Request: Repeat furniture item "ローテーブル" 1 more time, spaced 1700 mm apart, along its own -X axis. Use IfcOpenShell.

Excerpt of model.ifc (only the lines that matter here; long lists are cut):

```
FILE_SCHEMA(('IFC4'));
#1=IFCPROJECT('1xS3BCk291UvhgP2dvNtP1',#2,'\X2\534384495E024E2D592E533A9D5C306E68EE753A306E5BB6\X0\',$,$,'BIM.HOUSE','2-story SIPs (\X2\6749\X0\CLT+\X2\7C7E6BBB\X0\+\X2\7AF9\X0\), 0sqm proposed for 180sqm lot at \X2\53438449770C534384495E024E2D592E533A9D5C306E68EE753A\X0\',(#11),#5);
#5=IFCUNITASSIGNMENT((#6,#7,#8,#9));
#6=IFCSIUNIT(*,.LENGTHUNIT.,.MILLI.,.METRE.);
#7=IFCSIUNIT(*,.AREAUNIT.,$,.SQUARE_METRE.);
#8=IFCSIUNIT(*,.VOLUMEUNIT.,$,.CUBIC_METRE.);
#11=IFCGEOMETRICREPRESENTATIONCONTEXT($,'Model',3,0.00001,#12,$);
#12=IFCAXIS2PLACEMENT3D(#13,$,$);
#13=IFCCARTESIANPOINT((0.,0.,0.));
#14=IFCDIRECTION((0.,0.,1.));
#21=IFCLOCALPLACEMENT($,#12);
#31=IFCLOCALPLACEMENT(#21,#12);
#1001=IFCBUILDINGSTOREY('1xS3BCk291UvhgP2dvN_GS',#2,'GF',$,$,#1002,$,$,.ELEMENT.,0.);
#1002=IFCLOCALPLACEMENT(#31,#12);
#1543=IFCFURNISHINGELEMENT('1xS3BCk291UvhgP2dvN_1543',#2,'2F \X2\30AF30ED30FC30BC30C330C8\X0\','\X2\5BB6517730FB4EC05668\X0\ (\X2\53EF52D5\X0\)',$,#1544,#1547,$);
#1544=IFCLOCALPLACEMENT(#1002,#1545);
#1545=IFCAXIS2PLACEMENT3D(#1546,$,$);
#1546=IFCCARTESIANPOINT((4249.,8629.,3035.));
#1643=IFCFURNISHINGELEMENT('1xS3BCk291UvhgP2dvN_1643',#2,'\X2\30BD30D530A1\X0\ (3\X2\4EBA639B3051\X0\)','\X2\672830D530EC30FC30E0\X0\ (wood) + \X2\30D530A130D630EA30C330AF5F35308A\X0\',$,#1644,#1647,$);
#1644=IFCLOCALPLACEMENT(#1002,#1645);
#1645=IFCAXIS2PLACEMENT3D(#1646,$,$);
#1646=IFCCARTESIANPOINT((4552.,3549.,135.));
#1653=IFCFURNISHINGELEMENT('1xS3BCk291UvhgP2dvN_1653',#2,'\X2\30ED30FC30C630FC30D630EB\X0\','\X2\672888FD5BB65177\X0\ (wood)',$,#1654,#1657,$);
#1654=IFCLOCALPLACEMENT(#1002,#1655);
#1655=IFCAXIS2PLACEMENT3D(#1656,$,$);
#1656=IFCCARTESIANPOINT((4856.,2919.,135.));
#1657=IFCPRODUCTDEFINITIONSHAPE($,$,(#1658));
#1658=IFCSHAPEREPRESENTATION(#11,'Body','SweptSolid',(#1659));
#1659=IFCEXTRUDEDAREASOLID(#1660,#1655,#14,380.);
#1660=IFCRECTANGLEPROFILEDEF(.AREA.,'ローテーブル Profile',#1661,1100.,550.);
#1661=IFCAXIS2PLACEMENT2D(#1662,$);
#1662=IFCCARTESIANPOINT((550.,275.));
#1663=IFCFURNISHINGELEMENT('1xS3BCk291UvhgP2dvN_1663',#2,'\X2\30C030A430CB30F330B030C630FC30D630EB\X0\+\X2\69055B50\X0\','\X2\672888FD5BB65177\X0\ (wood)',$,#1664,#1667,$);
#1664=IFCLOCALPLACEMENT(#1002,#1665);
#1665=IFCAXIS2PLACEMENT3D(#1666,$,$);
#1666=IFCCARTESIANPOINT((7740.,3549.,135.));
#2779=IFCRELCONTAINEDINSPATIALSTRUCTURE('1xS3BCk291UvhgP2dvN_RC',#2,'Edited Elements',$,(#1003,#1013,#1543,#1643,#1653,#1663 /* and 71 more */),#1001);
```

```python
import ifcopenshell
import ifcopenshell.api.geometry
import ifcopenshell.api.root
import ifcopenshell.util.element
import ifcopenshell.util.placement
import ifcopenshell.util.unit

model = ifcopenshell.open("model.ifc")
unit_scale = ifcopenshell.util.unit.calculate_unit_scale(model)


def reuse_history(source, copy):
    """copy_class also copies each property set's owner history, people and application; keep the originals."""
    for rel in copy.IsDefinedBy:
        if rel.is_a("IfcRelDefinesByProperties") and (history := rel.RelatingPropertyDefinition.OwnerHistory):
            rel.RelatingPropertyDefinition.OwnerHistory = source.OwnerHistory
            ifcopenshell.util.element.remove_deep2(model, history)


source = model.by_guid("1xS3BCk291UvhgP2dvN_1653")
base = ifcopenshell.util.placement.get_local_placement(source.ObjectPlacement)
step = -base[:3, 0] * 1.7 / unit_scale

for i in range(1, 2):
    copy = ifcopenshell.api.root.copy_class(model, product=source)
    copy.Representation = ifcopenshell.util.element.copy_deep(
        model, source.Representation, exclude=["IfcGeometricRepresentationContext", "IfcRepresentationMap"]
    )
    reuse_history(source, copy)
    matrix = base.copy()
    matrix[:3, 3] += i * step
    print("added at", matrix[:3, 3].round(3) + 0.0)
    ifcopenshell.api.geometry.edit_object_placement(model, product=copy, matrix=matrix, is_si=False)

model.write("model-out.ifc")
```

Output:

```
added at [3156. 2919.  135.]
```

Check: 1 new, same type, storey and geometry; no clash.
